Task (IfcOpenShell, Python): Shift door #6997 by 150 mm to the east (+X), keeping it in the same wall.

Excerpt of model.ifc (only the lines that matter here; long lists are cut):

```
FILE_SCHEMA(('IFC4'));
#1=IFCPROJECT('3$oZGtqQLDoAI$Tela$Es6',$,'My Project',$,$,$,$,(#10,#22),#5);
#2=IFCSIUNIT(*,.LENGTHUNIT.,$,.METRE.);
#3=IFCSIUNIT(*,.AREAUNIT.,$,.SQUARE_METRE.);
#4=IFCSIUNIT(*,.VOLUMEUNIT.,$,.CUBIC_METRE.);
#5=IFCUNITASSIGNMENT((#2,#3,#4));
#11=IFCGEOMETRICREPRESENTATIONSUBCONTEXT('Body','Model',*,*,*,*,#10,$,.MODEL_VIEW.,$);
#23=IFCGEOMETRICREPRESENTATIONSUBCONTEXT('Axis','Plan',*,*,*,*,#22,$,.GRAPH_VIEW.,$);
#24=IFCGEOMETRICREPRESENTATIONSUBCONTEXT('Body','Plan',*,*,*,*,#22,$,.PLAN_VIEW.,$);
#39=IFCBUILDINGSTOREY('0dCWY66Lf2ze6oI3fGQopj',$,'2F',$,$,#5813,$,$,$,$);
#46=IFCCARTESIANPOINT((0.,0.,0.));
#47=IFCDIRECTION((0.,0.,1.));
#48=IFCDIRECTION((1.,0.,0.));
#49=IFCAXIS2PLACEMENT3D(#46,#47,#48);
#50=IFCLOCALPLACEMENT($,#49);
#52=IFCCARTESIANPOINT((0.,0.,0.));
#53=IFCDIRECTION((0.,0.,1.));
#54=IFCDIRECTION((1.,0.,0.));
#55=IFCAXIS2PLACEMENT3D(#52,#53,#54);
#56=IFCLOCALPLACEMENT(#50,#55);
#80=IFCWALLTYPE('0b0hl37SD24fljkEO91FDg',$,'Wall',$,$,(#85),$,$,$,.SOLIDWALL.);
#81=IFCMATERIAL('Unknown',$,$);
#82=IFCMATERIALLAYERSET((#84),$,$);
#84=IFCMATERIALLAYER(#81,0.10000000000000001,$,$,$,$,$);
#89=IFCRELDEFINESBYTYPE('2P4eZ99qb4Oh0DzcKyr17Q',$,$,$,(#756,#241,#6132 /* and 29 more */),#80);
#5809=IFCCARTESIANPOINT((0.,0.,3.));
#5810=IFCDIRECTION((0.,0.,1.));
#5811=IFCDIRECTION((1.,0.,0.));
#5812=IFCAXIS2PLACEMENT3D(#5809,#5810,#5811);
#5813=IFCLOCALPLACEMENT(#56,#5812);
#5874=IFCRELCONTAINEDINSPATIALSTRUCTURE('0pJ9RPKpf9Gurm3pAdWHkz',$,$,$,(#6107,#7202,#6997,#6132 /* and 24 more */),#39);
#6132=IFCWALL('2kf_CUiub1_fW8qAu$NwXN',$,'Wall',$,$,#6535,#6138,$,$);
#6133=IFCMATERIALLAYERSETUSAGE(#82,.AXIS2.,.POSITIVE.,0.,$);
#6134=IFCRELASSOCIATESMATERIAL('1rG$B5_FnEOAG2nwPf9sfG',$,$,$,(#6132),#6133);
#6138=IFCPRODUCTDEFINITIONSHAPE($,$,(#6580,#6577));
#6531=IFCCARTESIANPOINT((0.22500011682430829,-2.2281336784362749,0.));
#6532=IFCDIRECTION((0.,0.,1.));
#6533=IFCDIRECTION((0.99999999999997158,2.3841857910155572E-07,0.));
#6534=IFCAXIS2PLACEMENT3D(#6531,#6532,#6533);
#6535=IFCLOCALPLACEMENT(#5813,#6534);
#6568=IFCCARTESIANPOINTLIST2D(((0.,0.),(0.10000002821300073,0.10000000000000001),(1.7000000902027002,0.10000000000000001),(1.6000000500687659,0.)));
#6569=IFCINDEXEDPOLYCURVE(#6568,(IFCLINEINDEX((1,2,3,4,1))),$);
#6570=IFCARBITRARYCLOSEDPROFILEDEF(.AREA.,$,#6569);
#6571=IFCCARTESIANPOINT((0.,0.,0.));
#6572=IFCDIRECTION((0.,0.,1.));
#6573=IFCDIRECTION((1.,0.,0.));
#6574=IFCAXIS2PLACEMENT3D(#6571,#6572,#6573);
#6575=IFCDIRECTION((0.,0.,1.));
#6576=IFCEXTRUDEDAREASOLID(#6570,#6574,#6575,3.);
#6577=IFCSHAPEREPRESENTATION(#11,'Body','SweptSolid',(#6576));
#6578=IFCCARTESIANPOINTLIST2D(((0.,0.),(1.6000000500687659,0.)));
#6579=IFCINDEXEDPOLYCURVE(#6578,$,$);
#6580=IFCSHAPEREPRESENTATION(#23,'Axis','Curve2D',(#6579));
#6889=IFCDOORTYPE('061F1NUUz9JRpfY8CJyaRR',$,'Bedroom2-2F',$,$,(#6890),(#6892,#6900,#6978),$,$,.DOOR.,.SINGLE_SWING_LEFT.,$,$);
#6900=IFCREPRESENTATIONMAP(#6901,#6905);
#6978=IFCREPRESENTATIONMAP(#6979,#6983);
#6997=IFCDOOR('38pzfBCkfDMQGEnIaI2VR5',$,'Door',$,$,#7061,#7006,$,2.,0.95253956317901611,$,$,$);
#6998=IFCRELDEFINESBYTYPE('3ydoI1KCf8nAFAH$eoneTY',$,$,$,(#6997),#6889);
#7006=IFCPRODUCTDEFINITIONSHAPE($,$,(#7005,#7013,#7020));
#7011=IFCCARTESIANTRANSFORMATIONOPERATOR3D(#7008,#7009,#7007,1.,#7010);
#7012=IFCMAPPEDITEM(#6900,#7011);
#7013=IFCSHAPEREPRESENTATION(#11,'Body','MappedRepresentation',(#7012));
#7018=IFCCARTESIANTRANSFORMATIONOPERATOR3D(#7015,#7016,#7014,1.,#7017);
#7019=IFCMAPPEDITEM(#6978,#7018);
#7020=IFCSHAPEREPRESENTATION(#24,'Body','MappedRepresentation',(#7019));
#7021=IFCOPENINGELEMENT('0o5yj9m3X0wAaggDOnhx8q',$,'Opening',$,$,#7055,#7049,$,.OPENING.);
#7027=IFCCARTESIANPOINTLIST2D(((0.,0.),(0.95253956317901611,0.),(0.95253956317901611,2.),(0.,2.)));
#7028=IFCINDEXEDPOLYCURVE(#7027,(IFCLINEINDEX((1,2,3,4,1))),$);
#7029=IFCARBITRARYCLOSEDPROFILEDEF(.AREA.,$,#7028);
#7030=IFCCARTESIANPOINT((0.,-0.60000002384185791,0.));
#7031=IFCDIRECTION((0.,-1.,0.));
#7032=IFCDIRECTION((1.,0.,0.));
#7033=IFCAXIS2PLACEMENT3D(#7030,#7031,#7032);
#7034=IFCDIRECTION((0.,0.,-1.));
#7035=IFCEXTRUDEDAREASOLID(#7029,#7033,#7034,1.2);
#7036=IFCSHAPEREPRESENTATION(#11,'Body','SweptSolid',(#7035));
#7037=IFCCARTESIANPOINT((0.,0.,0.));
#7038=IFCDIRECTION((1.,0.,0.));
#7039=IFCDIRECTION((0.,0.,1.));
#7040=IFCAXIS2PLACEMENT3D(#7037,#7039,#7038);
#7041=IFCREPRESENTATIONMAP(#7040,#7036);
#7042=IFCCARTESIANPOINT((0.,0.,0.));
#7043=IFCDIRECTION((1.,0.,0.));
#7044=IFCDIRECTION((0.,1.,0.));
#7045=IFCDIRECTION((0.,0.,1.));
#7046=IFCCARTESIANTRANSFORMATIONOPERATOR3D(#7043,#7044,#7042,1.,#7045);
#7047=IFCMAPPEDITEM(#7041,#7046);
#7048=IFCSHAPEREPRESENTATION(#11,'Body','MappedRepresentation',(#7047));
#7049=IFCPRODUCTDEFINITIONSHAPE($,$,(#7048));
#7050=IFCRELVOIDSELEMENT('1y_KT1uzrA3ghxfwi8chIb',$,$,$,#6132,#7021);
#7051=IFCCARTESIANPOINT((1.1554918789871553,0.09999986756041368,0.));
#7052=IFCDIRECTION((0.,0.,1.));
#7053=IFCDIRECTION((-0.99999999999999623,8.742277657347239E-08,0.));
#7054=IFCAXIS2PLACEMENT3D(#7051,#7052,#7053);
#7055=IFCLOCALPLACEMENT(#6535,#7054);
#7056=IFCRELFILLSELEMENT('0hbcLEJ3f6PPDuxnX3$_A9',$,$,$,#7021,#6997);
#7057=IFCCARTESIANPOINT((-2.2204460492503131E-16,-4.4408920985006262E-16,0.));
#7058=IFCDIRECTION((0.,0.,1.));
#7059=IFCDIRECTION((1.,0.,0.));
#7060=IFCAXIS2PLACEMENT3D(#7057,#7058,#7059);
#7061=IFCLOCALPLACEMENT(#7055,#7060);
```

```python
import ifcopenshell
import ifcopenshell.api.geometry
import ifcopenshell.util.placement
import ifcopenshell.util.unit

model = ifcopenshell.open("model.ifc")
unit_scale = ifcopenshell.util.unit.calculate_unit_scale(model)

door = model.by_guid("38pzfBCkfDMQGEnIaI2VR5")
opening = door.FillsVoids[0].RelatingOpeningElement
wall = opening.VoidsElements[0].RelatingBuildingElement

wall_matrix = ifcopenshell.util.placement.get_local_placement(wall.ObjectPlacement)
shift = wall_matrix[:3, 0] * 0.15 / unit_scale
before = ifcopenshell.util.placement.get_local_placement(door.ObjectPlacement)[:3, 3].copy()

# The door is placed relative to its opening, so it follows when the opening moves.
matrix = ifcopenshell.util.placement.get_local_placement(opening.ObjectPlacement)
matrix[:3, 3] += shift
ifcopenshell.api.geometry.edit_object_placement(
    model, product=opening, matrix=matrix, is_si=False, should_transform_children=True
)

after = ifcopenshell.util.placement.get_local_placement(door.ObjectPlacement)[:3, 3]
print("door moved by", (after - before).round(3) + 0.0)

model.write("model_rev.ifc")
```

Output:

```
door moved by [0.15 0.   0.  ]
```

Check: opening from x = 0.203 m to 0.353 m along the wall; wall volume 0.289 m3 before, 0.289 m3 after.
